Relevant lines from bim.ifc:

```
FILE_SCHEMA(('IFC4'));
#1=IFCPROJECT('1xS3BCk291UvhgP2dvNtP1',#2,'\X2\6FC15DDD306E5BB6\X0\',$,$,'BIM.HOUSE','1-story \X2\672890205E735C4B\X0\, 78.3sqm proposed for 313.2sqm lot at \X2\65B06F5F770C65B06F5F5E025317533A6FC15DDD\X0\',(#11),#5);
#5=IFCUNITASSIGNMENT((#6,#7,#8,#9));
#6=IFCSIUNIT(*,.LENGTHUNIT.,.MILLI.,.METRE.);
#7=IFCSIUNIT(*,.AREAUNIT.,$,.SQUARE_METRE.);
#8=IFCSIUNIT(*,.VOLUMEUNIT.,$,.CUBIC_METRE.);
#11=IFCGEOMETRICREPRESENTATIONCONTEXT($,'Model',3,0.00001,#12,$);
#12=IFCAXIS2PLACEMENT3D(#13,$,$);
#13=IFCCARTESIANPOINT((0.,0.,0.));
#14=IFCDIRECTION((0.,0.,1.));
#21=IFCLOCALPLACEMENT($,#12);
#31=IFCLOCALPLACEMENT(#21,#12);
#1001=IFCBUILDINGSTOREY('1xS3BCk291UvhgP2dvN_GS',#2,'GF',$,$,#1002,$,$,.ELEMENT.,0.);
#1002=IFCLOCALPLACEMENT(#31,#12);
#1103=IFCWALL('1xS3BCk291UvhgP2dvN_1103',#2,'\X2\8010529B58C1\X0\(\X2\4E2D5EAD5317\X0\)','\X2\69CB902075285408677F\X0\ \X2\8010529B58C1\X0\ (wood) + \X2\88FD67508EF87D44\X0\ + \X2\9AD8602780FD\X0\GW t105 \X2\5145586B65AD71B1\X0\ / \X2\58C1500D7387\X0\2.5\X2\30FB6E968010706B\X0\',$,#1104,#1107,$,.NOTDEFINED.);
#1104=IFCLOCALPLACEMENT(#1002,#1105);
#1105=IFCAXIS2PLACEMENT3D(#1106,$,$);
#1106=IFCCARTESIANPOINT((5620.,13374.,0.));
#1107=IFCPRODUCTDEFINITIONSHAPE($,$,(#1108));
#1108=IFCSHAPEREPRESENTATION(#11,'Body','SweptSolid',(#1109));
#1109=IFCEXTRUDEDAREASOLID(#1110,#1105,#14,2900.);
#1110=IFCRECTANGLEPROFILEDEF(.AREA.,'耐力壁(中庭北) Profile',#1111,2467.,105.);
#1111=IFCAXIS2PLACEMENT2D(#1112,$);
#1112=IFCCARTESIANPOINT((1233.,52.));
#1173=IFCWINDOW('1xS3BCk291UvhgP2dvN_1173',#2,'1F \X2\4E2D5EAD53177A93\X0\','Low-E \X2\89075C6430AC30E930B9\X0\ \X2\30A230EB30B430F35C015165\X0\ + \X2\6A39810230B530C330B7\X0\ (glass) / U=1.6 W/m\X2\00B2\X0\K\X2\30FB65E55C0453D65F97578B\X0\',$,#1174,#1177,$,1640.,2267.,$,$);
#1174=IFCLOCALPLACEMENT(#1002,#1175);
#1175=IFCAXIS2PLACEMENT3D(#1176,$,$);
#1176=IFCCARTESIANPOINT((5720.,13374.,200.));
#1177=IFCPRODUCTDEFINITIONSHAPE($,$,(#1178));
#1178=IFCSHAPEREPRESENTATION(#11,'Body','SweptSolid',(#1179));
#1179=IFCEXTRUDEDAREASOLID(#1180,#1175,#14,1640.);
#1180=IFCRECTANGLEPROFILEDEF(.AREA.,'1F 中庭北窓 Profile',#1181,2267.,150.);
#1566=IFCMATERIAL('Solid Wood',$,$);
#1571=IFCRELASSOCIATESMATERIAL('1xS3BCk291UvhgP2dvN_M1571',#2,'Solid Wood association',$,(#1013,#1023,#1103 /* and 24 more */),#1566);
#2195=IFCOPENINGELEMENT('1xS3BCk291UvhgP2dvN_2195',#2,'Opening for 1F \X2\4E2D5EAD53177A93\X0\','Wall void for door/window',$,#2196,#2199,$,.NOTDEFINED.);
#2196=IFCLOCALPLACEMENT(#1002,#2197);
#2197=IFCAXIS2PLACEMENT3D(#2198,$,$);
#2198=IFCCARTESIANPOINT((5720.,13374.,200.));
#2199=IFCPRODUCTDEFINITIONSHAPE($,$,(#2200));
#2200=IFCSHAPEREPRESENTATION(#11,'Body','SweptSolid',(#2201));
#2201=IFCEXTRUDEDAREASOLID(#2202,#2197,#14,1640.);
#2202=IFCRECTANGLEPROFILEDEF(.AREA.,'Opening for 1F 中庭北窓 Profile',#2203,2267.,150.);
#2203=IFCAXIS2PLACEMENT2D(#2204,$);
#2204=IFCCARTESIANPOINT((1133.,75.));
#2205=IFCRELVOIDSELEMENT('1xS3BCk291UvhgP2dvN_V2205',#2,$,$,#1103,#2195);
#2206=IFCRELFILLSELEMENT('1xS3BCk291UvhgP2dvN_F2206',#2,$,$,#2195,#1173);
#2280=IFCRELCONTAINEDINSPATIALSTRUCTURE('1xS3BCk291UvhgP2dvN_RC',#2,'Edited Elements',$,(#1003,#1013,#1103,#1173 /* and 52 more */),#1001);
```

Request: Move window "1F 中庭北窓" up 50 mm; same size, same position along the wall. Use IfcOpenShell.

```python
import numpy as np
import ifcopenshell
import ifcopenshell.api.geometry
import ifcopenshell.util.placement
import ifcopenshell.util.unit

model = ifcopenshell.open("bim.ifc")
unit_scale = ifcopenshell.util.unit.calculate_unit_scale(model)

window = model.by_guid("1xS3BCk291UvhgP2dvN_1173")
opening = window.FillsVoids[0].RelatingOpeningElement
dz = 50.0

shift = np.array([0.0, 0.0, dz])
# The window is not placed relative to its opening, so move both.
for product in (opening, window):
    matrix = ifcopenshell.util.placement.get_local_placement(product.ObjectPlacement)
    matrix[:3, 3] += shift
    ifcopenshell.api.geometry.edit_object_placement(model, product=product, matrix=matrix, is_si=False)

print(f"moved by {dz * unit_scale:+.3f} m")

model.write("bim-out.ifc")
```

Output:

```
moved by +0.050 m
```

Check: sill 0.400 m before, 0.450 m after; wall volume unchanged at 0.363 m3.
